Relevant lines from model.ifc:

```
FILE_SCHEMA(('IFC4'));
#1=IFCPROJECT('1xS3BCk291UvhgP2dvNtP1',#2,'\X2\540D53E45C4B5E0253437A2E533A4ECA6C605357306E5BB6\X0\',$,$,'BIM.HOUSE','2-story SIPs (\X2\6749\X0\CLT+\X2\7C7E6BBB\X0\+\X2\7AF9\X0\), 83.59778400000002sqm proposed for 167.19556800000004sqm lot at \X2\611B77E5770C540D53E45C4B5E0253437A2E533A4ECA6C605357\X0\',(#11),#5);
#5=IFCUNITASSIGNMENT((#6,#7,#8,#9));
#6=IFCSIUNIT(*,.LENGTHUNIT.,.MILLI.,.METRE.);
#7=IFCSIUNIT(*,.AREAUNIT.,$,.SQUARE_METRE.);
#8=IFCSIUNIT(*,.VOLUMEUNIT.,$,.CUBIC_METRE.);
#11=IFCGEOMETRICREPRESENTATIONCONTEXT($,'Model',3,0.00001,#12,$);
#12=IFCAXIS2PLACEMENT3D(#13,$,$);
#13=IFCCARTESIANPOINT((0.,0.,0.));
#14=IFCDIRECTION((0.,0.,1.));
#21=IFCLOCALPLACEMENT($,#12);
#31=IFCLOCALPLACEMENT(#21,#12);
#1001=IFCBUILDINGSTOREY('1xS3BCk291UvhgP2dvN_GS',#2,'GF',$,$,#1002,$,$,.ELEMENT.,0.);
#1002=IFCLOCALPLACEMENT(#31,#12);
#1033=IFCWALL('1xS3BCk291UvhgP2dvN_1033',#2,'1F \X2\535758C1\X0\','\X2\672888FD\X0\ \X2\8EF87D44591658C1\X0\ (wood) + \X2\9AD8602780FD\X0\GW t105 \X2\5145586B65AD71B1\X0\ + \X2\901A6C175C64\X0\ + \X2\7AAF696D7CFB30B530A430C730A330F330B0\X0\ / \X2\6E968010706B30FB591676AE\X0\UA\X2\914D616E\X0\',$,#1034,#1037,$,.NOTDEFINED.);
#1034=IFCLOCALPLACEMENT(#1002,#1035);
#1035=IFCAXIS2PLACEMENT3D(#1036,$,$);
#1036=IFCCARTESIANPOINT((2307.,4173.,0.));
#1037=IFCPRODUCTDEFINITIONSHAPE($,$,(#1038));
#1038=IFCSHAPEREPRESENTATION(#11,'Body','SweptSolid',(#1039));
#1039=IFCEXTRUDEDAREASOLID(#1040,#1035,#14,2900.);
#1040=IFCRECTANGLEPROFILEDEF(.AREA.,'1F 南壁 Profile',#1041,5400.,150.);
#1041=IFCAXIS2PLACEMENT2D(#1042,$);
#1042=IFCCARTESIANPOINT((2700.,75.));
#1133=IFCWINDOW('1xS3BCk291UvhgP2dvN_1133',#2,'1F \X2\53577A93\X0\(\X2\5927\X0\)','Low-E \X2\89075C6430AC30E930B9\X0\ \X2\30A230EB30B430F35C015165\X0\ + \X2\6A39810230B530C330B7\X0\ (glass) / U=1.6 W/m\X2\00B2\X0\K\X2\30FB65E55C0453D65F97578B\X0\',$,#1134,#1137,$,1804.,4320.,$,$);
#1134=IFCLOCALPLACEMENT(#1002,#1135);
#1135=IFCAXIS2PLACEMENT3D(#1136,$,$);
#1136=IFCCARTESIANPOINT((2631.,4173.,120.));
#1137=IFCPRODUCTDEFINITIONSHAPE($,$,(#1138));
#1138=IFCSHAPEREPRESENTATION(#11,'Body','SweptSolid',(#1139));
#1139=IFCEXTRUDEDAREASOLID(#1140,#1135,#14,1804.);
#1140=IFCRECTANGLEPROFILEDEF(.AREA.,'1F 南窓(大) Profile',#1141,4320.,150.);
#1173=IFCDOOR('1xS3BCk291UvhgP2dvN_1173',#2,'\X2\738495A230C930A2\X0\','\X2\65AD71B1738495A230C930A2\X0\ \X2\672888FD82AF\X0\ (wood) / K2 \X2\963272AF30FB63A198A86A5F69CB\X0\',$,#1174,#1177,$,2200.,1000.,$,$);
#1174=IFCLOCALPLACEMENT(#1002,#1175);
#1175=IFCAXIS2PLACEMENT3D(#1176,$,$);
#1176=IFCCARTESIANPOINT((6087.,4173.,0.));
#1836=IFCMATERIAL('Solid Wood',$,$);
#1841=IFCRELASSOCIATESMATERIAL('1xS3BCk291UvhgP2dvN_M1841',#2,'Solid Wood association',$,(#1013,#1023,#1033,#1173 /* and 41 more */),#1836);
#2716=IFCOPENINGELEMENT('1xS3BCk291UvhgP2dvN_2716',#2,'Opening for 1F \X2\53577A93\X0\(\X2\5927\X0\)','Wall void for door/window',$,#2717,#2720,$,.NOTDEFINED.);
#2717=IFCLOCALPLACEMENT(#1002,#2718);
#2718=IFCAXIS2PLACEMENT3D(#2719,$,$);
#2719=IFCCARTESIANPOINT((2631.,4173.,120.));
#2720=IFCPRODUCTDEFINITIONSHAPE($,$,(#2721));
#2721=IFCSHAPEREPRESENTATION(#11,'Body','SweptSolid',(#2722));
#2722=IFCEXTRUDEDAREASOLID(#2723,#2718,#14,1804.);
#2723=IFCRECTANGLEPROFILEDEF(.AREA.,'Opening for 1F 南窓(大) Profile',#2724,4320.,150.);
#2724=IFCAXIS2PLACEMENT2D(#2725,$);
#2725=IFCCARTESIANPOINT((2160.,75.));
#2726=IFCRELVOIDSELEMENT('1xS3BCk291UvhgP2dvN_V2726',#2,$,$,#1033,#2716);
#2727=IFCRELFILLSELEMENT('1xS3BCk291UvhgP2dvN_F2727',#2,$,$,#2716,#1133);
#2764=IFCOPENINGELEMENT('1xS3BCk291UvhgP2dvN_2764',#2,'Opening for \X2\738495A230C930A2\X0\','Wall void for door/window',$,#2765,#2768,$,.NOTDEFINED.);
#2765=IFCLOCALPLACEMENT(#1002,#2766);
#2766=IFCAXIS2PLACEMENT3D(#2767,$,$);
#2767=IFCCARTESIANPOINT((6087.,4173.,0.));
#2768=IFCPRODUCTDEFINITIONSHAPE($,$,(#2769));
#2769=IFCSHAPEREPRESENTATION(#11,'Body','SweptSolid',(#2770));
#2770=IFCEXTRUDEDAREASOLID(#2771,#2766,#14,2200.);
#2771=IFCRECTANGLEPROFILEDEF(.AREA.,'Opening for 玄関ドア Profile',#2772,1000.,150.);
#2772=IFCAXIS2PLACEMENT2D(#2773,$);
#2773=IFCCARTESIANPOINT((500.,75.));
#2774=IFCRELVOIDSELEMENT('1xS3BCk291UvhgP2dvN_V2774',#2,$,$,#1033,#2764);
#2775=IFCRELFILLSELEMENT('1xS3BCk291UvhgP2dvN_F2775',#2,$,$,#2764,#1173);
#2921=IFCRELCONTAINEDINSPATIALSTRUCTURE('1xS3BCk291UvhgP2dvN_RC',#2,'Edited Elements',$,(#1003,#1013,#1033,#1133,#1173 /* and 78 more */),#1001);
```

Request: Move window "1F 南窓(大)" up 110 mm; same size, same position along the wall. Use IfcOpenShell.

```python
import numpy as np
import ifcopenshell
import ifcopenshell.api.geometry
import ifcopenshell.util.placement
import ifcopenshell.util.unit

model = ifcopenshell.open("model.ifc")
unit_scale = ifcopenshell.util.unit.calculate_unit_scale(model)

window = model.by_id(1133)
opening = window.FillsVoids[0].RelatingOpeningElement
dz = 110.0

shift = np.array([0.0, 0.0, dz])
# The window is not placed relative to its opening, so move both.
for product in (opening, window):
    matrix = ifcopenshell.util.placement.get_local_placement(product.ObjectPlacement)
    matrix[:3, 3] += shift
    ifcopenshell.api.geometry.edit_object_placement(model, product=product, matrix=matrix, is_si=False)

print(f"moved by {dz * unit_scale:+.3f} m")

model.write("model_edited.ifc")
```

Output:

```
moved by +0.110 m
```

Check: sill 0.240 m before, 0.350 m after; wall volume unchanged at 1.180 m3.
